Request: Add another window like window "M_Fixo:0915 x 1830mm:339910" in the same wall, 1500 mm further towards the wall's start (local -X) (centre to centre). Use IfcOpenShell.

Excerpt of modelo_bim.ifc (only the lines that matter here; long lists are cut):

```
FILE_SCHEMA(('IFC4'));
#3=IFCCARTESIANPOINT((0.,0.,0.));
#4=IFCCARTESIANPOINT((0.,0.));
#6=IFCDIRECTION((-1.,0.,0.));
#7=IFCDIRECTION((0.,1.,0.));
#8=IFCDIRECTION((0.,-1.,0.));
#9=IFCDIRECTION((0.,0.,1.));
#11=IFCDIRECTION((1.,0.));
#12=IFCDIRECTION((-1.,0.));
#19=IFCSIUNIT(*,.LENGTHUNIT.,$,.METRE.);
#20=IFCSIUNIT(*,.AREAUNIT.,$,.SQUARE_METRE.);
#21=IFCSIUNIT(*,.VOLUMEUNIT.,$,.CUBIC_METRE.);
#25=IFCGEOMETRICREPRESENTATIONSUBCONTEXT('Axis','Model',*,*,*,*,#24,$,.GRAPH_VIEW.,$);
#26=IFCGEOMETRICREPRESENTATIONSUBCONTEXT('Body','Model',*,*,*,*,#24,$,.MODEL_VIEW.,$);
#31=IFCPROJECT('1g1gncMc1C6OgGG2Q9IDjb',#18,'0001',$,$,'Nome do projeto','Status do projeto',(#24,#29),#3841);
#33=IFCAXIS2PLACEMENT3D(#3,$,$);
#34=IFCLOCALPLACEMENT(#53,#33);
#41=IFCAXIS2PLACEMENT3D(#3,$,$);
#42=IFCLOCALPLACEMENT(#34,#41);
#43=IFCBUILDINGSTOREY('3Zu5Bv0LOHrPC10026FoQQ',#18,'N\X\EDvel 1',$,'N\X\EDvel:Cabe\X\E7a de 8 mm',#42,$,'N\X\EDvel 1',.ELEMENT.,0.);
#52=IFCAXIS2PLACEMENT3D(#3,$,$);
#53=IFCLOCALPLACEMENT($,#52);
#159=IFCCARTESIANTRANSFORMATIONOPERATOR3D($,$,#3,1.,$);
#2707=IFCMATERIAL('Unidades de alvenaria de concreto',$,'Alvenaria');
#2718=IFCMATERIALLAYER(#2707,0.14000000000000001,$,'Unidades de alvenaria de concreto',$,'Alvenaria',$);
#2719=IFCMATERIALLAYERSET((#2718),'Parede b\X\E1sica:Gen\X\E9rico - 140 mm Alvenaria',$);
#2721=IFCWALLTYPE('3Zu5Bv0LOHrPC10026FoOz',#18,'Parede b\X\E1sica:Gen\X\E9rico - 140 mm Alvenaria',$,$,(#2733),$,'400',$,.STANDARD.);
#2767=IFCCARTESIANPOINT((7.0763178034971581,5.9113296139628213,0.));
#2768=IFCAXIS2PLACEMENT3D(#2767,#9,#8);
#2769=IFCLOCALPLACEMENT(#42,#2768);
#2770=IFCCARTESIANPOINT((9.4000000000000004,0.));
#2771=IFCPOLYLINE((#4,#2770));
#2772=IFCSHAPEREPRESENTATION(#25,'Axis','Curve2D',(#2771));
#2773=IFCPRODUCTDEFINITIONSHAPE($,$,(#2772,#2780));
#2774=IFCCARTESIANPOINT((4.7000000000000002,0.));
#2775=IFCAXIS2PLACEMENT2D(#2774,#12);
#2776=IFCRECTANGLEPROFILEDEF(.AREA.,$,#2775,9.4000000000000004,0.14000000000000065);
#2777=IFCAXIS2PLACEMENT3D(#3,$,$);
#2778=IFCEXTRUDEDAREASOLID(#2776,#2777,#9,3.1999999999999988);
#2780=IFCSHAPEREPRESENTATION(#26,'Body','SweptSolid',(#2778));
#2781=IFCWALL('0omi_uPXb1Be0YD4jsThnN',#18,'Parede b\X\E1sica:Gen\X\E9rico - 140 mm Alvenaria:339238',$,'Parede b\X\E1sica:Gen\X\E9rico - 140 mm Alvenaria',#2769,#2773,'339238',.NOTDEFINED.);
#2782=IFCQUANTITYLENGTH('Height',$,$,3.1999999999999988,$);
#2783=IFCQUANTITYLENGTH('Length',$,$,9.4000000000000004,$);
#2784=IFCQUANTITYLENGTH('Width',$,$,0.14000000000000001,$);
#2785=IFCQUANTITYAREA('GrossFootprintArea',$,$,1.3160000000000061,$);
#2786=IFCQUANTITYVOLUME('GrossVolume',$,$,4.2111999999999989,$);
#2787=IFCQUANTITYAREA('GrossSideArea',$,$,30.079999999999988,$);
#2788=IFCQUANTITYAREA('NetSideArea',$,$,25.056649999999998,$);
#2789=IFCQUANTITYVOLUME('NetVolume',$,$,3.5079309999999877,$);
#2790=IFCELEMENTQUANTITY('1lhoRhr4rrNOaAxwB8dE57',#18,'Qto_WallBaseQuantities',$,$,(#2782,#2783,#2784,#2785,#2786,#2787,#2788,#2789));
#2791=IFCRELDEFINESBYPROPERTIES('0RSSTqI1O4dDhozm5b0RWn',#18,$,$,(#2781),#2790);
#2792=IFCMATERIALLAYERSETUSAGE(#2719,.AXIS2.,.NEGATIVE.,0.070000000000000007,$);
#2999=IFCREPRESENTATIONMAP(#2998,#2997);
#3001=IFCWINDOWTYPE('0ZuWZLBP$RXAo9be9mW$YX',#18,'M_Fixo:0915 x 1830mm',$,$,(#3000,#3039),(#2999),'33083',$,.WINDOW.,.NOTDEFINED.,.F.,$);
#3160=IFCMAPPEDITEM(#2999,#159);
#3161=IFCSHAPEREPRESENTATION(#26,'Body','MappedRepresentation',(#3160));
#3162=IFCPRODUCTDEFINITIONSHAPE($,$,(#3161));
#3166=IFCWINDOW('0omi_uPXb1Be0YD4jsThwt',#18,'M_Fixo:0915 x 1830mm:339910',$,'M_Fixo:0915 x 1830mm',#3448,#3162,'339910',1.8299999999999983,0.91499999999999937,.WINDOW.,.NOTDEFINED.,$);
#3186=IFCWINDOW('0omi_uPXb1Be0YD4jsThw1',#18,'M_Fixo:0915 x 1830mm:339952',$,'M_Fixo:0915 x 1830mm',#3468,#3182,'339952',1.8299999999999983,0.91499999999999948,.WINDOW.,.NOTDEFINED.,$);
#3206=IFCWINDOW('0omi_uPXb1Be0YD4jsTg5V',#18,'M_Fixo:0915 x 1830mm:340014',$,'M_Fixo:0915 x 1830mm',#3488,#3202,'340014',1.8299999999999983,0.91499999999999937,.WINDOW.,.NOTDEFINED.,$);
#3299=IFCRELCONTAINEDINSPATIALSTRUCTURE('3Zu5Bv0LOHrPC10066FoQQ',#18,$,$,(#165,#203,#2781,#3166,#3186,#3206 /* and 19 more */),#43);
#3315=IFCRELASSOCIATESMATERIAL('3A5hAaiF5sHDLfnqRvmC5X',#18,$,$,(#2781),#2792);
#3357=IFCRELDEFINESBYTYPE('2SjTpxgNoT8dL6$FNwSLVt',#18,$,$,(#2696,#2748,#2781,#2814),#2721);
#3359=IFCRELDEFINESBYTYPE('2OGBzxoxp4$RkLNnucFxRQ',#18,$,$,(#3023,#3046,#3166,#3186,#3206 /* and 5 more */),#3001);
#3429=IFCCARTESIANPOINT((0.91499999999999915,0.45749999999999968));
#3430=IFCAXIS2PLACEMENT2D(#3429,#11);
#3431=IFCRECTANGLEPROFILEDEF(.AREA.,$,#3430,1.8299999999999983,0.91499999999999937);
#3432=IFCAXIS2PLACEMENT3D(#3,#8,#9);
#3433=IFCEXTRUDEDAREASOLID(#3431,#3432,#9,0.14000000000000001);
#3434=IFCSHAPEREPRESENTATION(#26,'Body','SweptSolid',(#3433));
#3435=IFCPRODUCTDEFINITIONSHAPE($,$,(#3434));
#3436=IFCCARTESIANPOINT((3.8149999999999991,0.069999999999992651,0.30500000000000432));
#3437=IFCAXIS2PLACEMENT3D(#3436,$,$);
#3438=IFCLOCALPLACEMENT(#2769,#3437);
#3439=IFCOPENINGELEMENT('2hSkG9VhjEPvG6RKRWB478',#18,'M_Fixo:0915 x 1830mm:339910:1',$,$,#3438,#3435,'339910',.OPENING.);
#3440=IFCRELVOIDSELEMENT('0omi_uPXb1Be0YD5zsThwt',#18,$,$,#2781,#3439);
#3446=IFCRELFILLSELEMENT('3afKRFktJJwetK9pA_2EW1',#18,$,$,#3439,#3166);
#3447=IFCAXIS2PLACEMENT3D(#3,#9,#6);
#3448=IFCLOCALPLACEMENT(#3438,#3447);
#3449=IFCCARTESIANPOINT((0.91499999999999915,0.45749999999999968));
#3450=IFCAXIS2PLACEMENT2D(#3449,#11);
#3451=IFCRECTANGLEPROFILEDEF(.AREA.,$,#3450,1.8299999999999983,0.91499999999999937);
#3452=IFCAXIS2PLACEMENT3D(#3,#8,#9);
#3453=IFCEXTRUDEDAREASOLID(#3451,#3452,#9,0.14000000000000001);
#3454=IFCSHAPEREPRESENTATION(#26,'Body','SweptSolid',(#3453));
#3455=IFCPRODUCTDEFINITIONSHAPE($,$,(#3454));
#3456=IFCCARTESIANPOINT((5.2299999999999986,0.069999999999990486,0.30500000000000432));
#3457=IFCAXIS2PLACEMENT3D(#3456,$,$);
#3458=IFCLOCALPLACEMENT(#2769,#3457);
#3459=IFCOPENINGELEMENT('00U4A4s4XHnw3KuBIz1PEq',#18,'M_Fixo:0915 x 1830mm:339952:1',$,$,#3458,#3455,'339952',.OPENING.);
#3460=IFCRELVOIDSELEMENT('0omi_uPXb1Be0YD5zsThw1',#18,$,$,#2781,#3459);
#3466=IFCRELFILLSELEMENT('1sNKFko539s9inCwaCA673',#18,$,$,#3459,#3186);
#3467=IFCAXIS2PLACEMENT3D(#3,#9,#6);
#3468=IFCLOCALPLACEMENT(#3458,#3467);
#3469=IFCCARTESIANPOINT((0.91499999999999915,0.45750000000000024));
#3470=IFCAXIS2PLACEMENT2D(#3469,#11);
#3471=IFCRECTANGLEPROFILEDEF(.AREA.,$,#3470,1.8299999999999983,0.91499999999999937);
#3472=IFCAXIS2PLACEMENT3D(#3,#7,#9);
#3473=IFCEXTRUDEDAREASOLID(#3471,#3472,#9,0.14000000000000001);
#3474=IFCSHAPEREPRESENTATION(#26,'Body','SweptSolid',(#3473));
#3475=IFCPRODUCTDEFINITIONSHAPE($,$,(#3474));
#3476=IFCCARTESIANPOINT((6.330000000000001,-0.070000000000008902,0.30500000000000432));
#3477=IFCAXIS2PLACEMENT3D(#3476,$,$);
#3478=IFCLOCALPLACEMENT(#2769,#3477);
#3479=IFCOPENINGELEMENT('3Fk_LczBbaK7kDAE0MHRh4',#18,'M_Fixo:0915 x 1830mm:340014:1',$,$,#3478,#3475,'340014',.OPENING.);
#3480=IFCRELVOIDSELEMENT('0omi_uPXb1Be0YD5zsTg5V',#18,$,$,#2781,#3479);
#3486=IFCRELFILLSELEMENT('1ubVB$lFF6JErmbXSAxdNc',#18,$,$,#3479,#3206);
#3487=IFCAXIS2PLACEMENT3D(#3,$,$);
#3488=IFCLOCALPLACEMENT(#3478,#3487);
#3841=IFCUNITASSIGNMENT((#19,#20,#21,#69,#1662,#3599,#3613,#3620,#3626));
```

```python
import ifcopenshell
import ifcopenshell.api.feature
import ifcopenshell.api.geometry
import ifcopenshell.api.pset
import ifcopenshell.api.root
import ifcopenshell.geom
import ifcopenshell.util.element
import ifcopenshell.util.placement
import ifcopenshell.util.shape
import ifcopenshell.util.unit

model = ifcopenshell.open("modelo_bim.ifc")
unit_scale = ifcopenshell.util.unit.calculate_unit_scale(model)
area_scale = ifcopenshell.util.unit.calculate_unit_scale(model, "AREAUNIT")
volume_scale = ifcopenshell.util.unit.calculate_unit_scale(model, "VOLUMEUNIT")
settings = ifcopenshell.geom.settings()


def volume(element):
    """Net volume in cubic metres, openings subtracted."""
    shape = ifcopenshell.geom.create_shape(settings, element)
    return ifcopenshell.util.shape.get_volume(shape.geometry)


def reuse_history(source, copy):
    """copy_class also copies each property set's owner history, people and application; keep the originals."""
    for rel in copy.IsDefinedBy:
        if rel.is_a("IfcRelDefinesByProperties") and (history := rel.RelatingPropertyDefinition.OwnerHistory):
            rel.RelatingPropertyDefinition.OwnerHistory = source.OwnerHistory
            ifcopenshell.util.element.remove_deep2(model, history)


window = model.by_guid("0omi_uPXb1Be0YD4jsThwt")
opening = window.FillsVoids[0].RelatingOpeningElement
wall = opening.VoidsElements[0].RelatingBuildingElement
before = volume(wall)
shift = ifcopenshell.util.placement.get_local_placement(wall.ObjectPlacement)[:3, 0] * -1.5 / unit_scale

# copy_class copies the void relationship, type, container and properties, but no geometry.
new_opening = ifcopenshell.api.root.copy_class(model, product=opening)
new_opening.Representation = ifcopenshell.util.element.copy_deep(
    model, opening.Representation, exclude=["IfcGeometricRepresentationContext", "IfcRepresentationMap"]
)
new_opening.Name = "M_Fixo:0915 x 1830mm"
new_opening.Tag = None
reuse_history(opening, new_opening)
new_window = ifcopenshell.api.root.copy_class(model, product=window)
new_window.Representation = ifcopenshell.util.element.copy_deep(
    model, window.Representation, exclude=["IfcGeometricRepresentationContext", "IfcRepresentationMap"]
)
new_window.Name = "M_Fixo:0915 x 1830mm"
new_window.Tag = None
reuse_history(window, new_window)
ifcopenshell.api.feature.add_filling(model, opening=new_opening, element=new_window)

for old, new in ((opening, new_opening), (window, new_window)):
    matrix = ifcopenshell.util.placement.get_local_placement(old.ObjectPlacement)
    matrix[:3, 3] += shift
    ifcopenshell.api.geometry.edit_object_placement(model, product=new, matrix=matrix, is_si=False)

after = volume(wall)
thickness = 0.14  # wall thickness in metres

# Update the wall's stored quantities.
qto = model.by_id(ifcopenshell.util.element.get_pset(wall, "Qto_WallBaseQuantities", should_inherit=False)["id"])
ifcopenshell.api.pset.edit_qto(model, qto=qto, properties={
    "NetSideArea": after / thickness / area_scale,
    "NetVolume": after / volume_scale,
})

print(f"wall volume {before:.3f} -> {after:.3f} m3")

model.write("modelo_bim_rev.ifc")
```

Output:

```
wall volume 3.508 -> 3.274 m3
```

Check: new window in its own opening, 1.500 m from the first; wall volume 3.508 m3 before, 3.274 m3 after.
